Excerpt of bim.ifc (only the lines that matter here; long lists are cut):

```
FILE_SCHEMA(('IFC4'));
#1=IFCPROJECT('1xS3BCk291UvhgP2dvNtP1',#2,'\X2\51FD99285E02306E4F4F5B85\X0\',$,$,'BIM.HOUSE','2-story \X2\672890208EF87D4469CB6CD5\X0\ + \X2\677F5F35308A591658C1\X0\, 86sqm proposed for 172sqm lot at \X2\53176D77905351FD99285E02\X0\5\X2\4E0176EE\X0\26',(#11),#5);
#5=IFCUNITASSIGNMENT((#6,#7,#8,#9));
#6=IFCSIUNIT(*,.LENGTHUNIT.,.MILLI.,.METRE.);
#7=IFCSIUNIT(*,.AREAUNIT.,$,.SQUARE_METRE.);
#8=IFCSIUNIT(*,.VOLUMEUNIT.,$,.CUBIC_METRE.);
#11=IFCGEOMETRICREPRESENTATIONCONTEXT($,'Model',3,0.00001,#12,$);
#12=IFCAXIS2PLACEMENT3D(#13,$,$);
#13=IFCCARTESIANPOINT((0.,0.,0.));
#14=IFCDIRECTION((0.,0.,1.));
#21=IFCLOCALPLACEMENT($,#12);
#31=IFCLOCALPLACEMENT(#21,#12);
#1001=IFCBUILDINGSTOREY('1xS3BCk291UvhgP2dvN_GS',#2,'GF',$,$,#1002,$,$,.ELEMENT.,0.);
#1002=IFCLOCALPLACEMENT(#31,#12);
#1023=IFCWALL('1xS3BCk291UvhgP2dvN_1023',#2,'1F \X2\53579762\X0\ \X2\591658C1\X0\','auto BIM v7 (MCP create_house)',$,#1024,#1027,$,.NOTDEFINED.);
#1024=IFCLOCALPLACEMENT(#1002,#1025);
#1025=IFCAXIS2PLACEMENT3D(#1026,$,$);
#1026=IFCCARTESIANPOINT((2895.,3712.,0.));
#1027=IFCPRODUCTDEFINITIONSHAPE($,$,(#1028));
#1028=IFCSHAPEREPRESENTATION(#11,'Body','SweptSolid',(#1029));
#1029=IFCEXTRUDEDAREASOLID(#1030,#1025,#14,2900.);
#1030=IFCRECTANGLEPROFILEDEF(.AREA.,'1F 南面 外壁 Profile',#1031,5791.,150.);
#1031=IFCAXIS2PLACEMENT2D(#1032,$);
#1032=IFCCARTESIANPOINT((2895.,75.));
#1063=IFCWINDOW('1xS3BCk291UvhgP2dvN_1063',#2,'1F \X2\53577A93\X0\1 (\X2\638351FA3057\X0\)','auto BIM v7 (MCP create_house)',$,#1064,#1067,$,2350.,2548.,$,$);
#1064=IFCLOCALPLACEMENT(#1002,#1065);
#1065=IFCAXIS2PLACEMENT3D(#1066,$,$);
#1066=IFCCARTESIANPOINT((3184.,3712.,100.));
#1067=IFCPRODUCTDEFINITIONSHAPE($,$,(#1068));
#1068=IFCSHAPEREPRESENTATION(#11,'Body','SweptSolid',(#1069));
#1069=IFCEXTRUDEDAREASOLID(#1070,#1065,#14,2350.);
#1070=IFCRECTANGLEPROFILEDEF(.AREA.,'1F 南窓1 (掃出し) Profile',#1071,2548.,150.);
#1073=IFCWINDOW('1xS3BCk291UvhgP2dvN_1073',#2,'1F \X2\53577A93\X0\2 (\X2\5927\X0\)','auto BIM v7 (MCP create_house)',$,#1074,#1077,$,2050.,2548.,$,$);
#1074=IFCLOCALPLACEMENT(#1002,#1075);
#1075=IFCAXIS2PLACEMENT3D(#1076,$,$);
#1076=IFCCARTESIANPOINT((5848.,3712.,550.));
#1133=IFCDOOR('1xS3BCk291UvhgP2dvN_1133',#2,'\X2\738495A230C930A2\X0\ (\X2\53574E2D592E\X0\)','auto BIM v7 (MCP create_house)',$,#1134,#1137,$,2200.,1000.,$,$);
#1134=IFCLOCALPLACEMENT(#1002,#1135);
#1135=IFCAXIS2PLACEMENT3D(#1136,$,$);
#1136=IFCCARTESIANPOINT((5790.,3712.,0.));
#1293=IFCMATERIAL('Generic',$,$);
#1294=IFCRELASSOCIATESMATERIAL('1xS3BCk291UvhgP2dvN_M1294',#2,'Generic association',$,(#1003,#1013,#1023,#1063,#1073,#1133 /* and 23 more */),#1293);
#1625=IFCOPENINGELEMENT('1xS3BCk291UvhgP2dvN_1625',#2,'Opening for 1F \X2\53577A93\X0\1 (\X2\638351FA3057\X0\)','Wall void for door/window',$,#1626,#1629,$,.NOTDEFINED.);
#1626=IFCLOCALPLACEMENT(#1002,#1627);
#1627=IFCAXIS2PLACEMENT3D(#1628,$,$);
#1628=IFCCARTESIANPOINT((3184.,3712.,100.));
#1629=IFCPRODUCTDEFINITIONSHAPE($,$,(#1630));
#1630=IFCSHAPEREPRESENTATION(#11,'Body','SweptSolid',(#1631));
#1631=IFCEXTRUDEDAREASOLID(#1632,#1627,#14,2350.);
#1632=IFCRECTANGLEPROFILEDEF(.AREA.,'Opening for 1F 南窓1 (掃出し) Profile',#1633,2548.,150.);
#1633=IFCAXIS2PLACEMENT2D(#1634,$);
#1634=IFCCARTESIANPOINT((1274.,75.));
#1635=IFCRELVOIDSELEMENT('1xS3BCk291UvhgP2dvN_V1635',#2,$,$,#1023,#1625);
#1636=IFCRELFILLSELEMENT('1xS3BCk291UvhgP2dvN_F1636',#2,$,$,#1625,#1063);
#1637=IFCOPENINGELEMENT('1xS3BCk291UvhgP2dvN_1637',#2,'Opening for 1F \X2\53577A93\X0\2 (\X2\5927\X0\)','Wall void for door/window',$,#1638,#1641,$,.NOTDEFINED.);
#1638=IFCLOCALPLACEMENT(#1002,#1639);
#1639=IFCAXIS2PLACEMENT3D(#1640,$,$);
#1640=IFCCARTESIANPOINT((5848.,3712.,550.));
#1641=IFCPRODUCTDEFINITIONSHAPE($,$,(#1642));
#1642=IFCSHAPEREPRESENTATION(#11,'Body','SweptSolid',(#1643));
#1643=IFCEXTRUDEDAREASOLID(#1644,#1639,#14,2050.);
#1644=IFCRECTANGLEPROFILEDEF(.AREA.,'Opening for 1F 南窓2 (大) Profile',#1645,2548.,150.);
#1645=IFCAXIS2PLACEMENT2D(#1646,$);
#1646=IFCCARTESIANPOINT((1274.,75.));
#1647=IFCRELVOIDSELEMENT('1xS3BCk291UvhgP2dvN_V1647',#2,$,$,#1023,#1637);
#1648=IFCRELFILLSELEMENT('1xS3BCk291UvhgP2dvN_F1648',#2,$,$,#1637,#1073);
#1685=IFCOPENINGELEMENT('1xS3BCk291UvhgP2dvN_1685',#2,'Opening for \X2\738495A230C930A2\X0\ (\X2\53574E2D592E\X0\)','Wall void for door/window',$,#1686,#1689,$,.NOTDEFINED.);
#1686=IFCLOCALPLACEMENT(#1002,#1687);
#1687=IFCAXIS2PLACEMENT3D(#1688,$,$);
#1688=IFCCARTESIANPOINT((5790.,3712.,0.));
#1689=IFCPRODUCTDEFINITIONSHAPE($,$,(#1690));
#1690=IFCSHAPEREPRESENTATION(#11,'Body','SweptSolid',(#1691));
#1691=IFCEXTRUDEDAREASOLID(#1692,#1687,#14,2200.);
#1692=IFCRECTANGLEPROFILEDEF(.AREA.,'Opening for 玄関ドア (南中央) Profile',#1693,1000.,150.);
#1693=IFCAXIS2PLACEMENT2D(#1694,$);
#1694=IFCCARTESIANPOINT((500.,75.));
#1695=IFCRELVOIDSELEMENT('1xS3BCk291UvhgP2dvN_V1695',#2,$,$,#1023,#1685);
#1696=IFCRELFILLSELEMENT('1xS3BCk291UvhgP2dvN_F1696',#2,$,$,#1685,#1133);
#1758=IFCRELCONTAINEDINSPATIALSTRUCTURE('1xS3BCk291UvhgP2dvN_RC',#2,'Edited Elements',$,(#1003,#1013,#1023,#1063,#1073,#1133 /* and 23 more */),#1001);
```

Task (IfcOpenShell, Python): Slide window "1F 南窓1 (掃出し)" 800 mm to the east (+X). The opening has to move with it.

```python
import ifcopenshell
import ifcopenshell.api.geometry
import ifcopenshell.util.placement

model = ifcopenshell.open("bim.ifc")

window = model.by_id(1063)
opening = window.FillsVoids[0].RelatingOpeningElement
wall = opening.VoidsElements[0].RelatingBuildingElement

wall_matrix = ifcopenshell.util.placement.get_local_placement(wall.ObjectPlacement)
shift = wall_matrix[:3, 0] * 800.0
before = ifcopenshell.util.placement.get_local_placement(window.ObjectPlacement)[:3, 3].copy()

# The window is not placed relative to its opening, so move both.
for product in (opening, window):
    matrix = ifcopenshell.util.placement.get_local_placement(product.ObjectPlacement)
    matrix[:3, 3] += shift
    ifcopenshell.api.geometry.edit_object_placement(model, product=product, matrix=matrix, is_si=False)

after = ifcopenshell.util.placement.get_local_placement(window.ObjectPlacement)[:3, 3]
print("window moved by", (after - before).round(3) + 0.0)

model.write("bim_updated.ifc")
```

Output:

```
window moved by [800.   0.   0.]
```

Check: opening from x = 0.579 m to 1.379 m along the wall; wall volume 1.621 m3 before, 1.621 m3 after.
